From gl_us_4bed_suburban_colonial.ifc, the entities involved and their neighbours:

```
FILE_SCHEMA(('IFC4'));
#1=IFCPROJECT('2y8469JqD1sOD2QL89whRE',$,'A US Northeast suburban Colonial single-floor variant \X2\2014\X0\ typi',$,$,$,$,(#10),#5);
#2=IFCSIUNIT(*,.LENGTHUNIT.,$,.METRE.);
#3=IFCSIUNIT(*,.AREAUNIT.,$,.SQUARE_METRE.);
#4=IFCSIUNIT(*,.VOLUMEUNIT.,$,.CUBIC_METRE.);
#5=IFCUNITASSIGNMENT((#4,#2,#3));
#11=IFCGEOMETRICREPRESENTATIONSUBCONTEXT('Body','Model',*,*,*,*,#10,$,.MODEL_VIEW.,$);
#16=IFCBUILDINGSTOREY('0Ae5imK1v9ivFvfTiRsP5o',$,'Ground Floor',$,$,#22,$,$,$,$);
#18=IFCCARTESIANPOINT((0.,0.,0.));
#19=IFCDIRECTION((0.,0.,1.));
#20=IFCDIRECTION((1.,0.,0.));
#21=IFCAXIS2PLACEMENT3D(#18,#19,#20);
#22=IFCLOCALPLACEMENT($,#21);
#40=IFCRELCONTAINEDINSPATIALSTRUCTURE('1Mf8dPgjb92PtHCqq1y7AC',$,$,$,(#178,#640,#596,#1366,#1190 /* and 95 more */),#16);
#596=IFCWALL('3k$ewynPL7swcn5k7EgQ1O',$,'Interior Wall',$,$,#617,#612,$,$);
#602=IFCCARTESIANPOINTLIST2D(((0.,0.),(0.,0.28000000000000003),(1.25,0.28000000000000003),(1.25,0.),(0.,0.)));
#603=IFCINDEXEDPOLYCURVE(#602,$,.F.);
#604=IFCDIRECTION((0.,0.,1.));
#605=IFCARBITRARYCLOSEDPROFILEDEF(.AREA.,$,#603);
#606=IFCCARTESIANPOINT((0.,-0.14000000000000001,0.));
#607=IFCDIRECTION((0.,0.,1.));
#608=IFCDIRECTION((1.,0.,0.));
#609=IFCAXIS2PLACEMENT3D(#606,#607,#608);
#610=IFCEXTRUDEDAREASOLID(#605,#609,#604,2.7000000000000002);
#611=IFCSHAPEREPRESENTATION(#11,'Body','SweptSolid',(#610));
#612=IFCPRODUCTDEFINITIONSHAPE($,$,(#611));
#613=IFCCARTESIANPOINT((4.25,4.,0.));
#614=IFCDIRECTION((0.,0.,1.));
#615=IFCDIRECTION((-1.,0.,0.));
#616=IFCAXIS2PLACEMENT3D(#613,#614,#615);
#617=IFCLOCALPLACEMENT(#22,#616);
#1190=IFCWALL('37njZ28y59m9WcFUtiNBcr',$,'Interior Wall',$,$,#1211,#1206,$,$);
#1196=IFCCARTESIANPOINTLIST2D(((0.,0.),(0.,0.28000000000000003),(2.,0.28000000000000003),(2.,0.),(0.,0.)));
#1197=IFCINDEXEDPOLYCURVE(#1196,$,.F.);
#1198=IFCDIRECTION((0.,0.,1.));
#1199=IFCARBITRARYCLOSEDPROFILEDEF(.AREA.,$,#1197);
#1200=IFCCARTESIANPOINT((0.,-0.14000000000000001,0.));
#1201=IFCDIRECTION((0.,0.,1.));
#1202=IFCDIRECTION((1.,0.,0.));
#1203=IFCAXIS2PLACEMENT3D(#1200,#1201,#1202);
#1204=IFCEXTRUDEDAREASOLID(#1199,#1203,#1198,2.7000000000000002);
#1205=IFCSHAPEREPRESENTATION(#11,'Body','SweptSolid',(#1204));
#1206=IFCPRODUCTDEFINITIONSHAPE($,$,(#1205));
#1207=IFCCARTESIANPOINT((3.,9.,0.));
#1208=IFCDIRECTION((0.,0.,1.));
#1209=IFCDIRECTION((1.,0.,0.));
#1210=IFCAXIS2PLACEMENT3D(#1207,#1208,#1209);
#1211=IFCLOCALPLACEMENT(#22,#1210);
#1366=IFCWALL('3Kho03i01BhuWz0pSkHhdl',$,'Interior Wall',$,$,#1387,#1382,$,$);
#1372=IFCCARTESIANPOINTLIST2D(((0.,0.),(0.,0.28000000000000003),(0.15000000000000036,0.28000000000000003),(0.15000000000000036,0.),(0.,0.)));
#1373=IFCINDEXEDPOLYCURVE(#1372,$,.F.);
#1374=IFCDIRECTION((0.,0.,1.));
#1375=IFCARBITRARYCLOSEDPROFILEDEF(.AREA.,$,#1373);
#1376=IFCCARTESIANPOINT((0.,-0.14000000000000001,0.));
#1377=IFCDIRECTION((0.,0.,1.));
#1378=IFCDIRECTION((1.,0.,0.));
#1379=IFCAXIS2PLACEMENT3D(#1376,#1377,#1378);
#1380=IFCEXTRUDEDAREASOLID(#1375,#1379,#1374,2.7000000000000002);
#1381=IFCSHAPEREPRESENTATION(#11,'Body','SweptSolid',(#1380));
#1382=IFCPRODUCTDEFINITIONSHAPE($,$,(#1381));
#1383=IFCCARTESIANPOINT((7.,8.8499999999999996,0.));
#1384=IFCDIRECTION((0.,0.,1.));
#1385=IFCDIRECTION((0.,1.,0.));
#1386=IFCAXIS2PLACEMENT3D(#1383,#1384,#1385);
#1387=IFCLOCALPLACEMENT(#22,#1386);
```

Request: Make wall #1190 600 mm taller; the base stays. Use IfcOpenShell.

```python
import ifcopenshell
import ifcopenshell.geom
import ifcopenshell.util.representation
import ifcopenshell.util.shape

model = ifcopenshell.open("gl_us_4bed_suburban_colonial.ifc")
settings = ifcopenshell.geom.settings()


def volume(element):
    """Net volume in cubic metres, openings subtracted."""
    shape = ifcopenshell.geom.create_shape(settings, element)
    return ifcopenshell.util.shape.get_volume(shape.geometry)


wall = model.by_id(1190)
before = volume(wall)

body = ifcopenshell.util.representation.get_representation(wall, "Model", "Body")
solid = body.Items[0]
old_height = solid.Depth
solid.Depth += 0.6
after = volume(wall)

print(f"height {old_height:g} -> {solid.Depth:g}, volume {before:.3f} -> {after:.3f} m3")

model.write("gl_us_4bed_suburban_colonial_v2.ifc")
```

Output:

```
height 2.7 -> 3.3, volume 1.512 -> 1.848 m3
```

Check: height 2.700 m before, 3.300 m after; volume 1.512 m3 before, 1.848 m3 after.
